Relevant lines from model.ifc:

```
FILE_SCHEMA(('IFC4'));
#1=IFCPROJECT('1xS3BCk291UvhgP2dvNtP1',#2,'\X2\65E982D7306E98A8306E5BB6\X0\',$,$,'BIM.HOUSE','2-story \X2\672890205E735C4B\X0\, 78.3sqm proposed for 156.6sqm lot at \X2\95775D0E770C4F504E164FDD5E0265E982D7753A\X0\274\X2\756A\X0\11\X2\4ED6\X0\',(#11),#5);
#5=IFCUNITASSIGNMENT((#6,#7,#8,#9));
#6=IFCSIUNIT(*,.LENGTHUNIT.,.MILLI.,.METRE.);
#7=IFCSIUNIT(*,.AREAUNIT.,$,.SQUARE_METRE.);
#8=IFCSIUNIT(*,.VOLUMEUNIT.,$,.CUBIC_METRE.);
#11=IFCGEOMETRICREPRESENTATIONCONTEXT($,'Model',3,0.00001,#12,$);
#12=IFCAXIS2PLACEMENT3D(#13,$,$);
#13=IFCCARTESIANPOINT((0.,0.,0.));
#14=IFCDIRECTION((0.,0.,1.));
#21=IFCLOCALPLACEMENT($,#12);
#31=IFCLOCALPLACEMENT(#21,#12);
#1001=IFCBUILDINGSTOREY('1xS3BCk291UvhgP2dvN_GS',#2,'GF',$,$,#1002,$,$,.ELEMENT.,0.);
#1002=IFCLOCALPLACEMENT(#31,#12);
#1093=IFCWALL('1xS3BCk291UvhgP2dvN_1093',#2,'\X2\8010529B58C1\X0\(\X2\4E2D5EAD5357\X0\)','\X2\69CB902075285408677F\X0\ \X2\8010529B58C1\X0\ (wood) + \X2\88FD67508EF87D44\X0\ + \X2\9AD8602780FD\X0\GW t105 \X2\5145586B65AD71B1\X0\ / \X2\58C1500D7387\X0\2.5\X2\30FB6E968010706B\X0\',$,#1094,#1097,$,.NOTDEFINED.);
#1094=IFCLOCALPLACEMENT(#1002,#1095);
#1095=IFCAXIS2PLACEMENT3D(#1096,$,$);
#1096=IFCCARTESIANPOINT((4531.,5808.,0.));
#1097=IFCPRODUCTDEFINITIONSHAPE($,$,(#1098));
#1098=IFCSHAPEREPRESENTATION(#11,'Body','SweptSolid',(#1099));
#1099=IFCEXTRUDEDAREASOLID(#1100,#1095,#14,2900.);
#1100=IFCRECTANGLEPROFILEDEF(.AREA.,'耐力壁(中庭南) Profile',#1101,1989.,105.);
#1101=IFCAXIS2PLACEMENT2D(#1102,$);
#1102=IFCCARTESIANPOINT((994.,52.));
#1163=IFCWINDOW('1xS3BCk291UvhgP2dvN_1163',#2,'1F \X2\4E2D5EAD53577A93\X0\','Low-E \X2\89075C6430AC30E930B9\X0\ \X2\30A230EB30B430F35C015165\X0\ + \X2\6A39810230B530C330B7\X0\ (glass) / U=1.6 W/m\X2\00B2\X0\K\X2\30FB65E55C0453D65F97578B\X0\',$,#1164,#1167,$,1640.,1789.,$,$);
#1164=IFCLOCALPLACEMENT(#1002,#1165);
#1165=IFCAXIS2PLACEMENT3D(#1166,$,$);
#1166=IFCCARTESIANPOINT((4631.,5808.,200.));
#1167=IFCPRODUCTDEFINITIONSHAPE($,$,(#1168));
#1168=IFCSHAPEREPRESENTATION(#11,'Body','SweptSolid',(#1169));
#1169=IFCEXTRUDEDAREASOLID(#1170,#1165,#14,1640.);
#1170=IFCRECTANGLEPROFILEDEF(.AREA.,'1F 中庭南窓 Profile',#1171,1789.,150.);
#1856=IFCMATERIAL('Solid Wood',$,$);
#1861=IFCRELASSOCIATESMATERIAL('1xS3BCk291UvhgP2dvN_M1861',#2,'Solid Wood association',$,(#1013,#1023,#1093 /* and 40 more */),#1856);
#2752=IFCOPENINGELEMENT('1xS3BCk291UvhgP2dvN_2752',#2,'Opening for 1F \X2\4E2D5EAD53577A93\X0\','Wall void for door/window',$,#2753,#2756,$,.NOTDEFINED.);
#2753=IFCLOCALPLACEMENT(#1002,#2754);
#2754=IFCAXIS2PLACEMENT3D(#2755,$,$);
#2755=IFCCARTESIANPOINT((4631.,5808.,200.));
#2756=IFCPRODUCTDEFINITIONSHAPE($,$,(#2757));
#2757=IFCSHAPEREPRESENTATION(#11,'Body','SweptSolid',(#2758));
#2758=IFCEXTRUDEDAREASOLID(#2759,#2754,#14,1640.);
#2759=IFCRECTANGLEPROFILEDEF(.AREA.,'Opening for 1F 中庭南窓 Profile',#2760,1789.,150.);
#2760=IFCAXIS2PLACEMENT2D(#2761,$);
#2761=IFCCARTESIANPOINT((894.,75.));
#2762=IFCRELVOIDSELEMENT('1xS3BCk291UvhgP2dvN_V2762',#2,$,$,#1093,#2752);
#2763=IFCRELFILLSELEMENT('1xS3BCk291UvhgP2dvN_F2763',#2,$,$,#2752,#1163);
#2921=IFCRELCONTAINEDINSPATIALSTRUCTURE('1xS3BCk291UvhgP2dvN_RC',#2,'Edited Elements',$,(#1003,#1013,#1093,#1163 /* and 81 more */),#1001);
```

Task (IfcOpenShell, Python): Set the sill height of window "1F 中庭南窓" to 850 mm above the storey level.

```python
import numpy as np
import ifcopenshell
import ifcopenshell.api.geometry
import ifcopenshell.geom
import ifcopenshell.util.element
import ifcopenshell.util.placement
import ifcopenshell.util.shape
import ifcopenshell.util.unit

model = ifcopenshell.open("model.ifc")
unit_scale = ifcopenshell.util.unit.calculate_unit_scale(model)

window = model.by_guid("1xS3BCk291UvhgP2dvN_1163")
opening = window.FillsVoids[0].RelatingOpeningElement
storey = ifcopenshell.util.element.get_container(window, ifc_class="IfcBuildingStorey")
level = ifcopenshell.util.placement.get_local_placement(storey.ObjectPlacement)[2, 3]

# The opening's origin need not be at the sill, so measure its lowest point.
shape = ifcopenshell.geom.create_shape(ifcopenshell.geom.settings(), opening)
bottom = ifcopenshell.util.shape.get_shape_bottom_elevation(shape, shape.geometry) / unit_scale
dz = level + 0.85 / unit_scale - bottom

shift = np.array([0.0, 0.0, dz])
# The window is not placed relative to its opening, so move both.
for product in (opening, window):
    matrix = ifcopenshell.util.placement.get_local_placement(product.ObjectPlacement)
    matrix[:3, 3] += shift
    ifcopenshell.api.geometry.edit_object_placement(model, product=product, matrix=matrix, is_si=False)

print(f"moved by {dz * unit_scale:+.3f} m")

model.write("model_edited.ifc")
```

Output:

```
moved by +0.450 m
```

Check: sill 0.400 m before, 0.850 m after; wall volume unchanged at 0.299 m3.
